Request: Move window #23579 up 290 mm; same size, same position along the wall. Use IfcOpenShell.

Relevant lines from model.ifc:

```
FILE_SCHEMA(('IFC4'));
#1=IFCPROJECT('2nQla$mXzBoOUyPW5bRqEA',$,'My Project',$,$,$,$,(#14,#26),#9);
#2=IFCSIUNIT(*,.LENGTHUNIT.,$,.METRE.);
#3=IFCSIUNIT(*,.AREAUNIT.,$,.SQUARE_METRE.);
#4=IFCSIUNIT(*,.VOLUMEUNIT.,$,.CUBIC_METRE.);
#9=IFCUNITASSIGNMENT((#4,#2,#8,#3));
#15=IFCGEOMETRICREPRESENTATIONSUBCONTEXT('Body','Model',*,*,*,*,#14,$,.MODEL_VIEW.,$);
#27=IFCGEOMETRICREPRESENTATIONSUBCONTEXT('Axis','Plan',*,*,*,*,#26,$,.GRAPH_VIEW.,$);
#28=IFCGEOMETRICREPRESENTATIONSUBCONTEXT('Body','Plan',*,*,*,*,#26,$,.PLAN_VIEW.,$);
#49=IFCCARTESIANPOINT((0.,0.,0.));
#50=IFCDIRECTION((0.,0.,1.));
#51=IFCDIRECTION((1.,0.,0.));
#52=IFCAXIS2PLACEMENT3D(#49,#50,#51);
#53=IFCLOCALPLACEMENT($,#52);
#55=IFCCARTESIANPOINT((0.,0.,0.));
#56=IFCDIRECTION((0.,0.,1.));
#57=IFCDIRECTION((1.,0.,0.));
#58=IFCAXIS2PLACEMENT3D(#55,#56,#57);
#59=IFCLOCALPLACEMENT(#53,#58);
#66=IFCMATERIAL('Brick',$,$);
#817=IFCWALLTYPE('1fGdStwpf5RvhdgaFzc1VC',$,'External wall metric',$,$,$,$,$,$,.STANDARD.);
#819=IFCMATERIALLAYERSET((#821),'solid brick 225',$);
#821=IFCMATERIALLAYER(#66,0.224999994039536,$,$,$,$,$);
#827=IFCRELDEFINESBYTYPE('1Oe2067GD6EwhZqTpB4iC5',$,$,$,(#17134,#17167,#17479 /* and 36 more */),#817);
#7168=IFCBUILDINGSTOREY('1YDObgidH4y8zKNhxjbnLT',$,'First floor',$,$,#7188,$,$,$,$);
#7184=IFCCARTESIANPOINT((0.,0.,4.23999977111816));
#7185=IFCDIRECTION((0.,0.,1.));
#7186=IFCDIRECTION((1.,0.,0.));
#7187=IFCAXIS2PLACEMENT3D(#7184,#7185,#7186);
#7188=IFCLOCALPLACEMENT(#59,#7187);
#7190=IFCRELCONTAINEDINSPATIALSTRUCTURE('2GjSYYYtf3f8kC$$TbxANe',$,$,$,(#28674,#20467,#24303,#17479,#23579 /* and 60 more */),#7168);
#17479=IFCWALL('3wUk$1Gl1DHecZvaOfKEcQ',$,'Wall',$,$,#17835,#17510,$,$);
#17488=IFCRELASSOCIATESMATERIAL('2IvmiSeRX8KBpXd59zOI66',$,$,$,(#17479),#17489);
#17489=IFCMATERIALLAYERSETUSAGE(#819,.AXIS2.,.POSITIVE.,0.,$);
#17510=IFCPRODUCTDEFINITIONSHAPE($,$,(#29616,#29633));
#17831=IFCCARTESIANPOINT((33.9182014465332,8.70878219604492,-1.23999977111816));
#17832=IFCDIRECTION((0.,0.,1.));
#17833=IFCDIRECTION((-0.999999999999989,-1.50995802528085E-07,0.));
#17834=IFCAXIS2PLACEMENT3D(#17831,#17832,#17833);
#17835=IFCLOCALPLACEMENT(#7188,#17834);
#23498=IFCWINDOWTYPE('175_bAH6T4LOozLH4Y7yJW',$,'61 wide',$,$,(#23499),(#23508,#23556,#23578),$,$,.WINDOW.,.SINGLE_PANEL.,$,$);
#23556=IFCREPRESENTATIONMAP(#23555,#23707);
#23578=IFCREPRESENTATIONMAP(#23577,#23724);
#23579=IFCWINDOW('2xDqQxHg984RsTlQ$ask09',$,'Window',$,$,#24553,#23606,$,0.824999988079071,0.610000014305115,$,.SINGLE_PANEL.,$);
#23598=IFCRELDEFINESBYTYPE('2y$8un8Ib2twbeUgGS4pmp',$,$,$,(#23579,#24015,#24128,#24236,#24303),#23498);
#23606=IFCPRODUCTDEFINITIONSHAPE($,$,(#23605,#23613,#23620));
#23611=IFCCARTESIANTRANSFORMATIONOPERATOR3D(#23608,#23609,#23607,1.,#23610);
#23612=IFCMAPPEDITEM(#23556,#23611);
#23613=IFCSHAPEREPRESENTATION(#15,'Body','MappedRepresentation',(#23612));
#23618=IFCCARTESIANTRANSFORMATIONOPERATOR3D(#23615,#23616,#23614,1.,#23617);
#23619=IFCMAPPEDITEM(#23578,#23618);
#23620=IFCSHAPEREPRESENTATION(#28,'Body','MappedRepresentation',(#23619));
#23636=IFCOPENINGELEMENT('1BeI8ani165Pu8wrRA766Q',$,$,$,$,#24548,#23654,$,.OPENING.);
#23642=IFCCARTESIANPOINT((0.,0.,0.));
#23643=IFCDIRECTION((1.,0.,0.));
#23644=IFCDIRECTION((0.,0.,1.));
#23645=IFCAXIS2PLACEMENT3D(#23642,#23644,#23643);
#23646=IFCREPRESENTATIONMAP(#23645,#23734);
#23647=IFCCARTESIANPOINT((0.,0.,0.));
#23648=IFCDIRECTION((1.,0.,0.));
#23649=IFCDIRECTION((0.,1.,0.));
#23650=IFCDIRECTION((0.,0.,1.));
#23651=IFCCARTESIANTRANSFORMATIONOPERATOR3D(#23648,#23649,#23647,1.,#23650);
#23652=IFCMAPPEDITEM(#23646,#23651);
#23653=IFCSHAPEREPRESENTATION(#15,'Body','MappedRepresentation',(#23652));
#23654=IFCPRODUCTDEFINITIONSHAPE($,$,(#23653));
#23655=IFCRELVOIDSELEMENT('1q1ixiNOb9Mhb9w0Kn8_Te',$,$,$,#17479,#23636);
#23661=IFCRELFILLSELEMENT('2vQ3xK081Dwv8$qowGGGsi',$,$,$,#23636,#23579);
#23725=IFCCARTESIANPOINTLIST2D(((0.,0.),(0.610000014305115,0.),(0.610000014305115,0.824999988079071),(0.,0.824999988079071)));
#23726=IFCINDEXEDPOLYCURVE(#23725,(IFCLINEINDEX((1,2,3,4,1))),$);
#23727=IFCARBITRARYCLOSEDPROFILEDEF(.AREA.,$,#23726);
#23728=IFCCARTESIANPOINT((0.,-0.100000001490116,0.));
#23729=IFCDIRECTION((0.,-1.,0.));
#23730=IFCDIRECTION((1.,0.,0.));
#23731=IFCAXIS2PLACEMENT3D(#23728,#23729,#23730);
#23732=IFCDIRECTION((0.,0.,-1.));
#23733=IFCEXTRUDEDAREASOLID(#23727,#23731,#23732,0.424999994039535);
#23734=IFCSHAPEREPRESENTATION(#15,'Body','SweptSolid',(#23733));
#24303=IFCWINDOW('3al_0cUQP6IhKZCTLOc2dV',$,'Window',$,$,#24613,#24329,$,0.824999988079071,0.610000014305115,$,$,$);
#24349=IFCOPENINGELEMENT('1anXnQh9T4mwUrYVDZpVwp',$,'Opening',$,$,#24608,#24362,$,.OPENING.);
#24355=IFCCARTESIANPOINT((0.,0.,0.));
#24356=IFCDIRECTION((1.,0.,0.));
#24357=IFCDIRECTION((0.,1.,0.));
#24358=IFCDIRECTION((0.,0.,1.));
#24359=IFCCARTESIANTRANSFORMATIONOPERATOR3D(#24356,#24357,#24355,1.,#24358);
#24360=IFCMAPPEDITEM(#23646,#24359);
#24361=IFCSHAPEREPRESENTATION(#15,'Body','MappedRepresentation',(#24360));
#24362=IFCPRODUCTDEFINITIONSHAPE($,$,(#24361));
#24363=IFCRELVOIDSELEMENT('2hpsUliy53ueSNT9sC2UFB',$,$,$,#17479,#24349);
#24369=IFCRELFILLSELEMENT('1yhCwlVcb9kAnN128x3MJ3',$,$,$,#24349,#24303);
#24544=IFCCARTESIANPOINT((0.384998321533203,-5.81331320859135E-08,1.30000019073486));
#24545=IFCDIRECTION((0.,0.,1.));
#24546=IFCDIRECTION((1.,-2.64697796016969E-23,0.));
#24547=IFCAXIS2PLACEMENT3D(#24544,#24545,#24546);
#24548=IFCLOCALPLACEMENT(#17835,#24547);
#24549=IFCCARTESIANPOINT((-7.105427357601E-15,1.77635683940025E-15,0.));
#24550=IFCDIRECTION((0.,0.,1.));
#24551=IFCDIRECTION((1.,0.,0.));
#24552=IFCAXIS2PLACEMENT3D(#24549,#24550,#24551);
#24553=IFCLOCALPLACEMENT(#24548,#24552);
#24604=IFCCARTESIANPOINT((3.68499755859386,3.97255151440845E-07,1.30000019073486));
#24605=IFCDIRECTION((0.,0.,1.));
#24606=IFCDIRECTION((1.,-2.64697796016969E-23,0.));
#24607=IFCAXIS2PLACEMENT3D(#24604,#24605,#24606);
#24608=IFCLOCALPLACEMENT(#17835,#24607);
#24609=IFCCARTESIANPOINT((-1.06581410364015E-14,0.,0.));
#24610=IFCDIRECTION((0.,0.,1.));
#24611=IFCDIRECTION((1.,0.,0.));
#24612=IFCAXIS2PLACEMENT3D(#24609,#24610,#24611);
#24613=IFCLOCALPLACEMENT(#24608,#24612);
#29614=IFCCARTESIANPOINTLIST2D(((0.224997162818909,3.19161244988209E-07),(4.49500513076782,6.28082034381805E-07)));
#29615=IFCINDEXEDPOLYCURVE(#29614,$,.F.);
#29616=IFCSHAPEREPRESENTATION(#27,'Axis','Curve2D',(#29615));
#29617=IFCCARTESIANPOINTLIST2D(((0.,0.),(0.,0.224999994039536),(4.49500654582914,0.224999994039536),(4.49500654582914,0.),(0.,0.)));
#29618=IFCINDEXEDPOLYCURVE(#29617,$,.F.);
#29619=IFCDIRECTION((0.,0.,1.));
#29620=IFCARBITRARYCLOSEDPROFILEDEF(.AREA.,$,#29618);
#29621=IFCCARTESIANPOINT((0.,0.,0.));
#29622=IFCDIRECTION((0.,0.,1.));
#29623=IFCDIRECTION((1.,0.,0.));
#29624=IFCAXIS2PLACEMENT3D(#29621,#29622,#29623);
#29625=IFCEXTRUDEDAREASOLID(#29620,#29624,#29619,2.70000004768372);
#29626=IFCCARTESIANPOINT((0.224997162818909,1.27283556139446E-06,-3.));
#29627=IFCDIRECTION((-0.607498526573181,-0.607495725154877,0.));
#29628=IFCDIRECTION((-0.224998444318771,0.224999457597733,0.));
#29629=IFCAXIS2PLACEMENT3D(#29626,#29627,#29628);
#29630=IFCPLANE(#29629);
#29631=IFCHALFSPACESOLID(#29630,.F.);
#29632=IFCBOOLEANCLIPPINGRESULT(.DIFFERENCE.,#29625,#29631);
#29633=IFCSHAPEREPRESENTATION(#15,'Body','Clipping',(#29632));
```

```python
import numpy as np
import ifcopenshell
import ifcopenshell.api.geometry
import ifcopenshell.util.placement
import ifcopenshell.util.unit

model = ifcopenshell.open("model.ifc")
unit_scale = ifcopenshell.util.unit.calculate_unit_scale(model)

window = model.by_id(23579)
opening = window.FillsVoids[0].RelatingOpeningElement
dz = 0.29 / unit_scale

shift = np.array([0.0, 0.0, dz])
# The window is placed relative to its opening, so it follows when the opening moves.
matrix = ifcopenshell.util.placement.get_local_placement(opening.ObjectPlacement)
matrix[:3, 3] += shift
ifcopenshell.api.geometry.edit_object_placement(
    model, product=opening, matrix=matrix, is_si=False, should_transform_children=True
)

print(f"moved by {dz * unit_scale:+.3f} m")

model.write("model_rev.ifc")
```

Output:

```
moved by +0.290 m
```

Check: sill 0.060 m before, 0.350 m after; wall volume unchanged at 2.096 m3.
